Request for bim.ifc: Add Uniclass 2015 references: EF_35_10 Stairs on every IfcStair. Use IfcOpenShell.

First a look at what the model holds.

```python
import ifcopenshell

model = ifcopenshell.open("bim.ifc")
print(model.schema)
print("classifications:", [c.Name for c in model.by_type("IfcClassification")])
for ifc_class in ("IfcDoor", "IfcRoof", "IfcStair", "IfcWall", "IfcWindow"):
    print(ifc_class, len(model.by_type(ifc_class)))
```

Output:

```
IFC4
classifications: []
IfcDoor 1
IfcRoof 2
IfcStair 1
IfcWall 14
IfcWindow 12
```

```python
import ifcopenshell
import ifcopenshell.api.classification

model = ifcopenshell.open("bim.ifc")

system = ifcopenshell.api.classification.add_classification(model, classification="Uniclass 2015")

codes = {
    "IfcStair": ("EF_35_10", "Stairs"),
}
for ifc_class, (code, name) in codes.items():
    products = model.by_type(ifc_class)
    ifcopenshell.api.classification.add_reference(
        model, products=products, classification=system, identification=code, name=name
    )
    print(code, len(products))

model.write("bim-out.ifc")
```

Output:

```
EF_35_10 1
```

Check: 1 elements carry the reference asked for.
